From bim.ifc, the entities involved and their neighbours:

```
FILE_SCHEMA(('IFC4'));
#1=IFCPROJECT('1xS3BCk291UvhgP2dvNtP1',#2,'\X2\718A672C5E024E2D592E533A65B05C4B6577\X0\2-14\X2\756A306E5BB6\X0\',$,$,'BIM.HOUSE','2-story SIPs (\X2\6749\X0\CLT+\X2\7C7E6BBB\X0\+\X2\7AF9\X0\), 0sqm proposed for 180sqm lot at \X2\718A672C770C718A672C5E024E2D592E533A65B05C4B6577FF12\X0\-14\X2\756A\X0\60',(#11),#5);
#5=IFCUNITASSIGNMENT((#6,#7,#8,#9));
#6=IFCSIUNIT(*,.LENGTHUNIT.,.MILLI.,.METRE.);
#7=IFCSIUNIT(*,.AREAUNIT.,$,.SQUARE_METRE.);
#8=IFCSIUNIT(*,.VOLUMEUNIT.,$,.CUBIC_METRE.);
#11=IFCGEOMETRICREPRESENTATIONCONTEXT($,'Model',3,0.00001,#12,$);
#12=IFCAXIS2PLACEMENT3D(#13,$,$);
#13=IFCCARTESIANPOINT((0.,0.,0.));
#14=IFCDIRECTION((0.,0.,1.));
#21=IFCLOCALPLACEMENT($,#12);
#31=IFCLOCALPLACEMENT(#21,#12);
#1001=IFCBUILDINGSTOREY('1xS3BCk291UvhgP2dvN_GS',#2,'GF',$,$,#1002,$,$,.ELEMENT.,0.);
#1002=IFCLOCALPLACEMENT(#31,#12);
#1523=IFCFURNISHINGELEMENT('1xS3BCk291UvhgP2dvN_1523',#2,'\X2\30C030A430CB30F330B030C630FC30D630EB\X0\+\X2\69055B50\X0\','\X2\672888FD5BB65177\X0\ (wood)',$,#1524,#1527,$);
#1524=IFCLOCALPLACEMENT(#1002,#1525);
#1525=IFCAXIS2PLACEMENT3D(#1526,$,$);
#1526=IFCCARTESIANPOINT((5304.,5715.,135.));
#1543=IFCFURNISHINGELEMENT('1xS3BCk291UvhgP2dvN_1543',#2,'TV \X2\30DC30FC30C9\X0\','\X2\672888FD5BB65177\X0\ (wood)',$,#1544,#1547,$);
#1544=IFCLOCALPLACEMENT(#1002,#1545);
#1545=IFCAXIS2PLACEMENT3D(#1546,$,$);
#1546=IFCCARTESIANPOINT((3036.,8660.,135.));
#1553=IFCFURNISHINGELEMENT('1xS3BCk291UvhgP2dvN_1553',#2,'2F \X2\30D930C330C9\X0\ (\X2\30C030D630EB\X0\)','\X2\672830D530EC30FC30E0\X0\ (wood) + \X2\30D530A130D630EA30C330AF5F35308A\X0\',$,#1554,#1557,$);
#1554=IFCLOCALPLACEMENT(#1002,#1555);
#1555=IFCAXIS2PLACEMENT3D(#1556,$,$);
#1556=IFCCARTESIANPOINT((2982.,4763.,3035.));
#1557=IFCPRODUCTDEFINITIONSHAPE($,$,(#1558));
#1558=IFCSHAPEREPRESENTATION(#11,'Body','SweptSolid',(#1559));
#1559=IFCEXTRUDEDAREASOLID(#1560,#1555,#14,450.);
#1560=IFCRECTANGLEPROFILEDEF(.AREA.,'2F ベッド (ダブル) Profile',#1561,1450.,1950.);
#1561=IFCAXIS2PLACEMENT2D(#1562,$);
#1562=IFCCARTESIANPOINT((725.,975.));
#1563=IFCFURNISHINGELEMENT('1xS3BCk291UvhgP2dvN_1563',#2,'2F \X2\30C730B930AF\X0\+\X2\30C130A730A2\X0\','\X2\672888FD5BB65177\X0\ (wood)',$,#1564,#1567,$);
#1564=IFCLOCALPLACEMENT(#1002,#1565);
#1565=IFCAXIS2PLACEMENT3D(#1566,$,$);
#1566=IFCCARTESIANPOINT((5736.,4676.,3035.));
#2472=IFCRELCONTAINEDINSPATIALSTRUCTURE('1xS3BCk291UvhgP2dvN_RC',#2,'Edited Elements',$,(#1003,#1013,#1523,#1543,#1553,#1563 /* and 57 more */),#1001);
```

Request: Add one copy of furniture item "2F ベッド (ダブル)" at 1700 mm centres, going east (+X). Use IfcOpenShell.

```python
import numpy as np
import ifcopenshell
import ifcopenshell.api.geometry
import ifcopenshell.api.root
import ifcopenshell.util.element
import ifcopenshell.util.placement

model = ifcopenshell.open("bim.ifc")


def reuse_history(source, copy):
    """copy_class also copies each property set's owner history, people and application; keep the originals."""
    for rel in copy.IsDefinedBy:
        if rel.is_a("IfcRelDefinesByProperties") and (history := rel.RelatingPropertyDefinition.OwnerHistory):
            rel.RelatingPropertyDefinition.OwnerHistory = source.OwnerHistory
            ifcopenshell.util.element.remove_deep2(model, history)


source = model.by_guid("1xS3BCk291UvhgP2dvN_1553")
base = ifcopenshell.util.placement.get_local_placement(source.ObjectPlacement)
step = np.array([1.0, 0.0, 0.0]) * 1700.0

for i in range(1, 2):
    copy = ifcopenshell.api.root.copy_class(model, product=source)
    copy.Representation = ifcopenshell.util.element.copy_deep(
        model, source.Representation, exclude=["IfcGeometricRepresentationContext", "IfcRepresentationMap"]
    )
    reuse_history(source, copy)
    matrix = base.copy()
    matrix[:3, 3] += i * step
    print("added at", matrix[:3, 3].round(3) + 0.0)
    ifcopenshell.api.geometry.edit_object_placement(model, product=copy, matrix=matrix, is_si=False)

model.write("bim_v2.ifc")
```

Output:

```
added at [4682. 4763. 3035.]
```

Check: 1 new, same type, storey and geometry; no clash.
